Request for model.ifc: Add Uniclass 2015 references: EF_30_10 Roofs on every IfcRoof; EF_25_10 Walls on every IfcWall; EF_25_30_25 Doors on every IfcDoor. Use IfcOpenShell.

First a look at what the model holds.

```python
import ifcopenshell

model = ifcopenshell.open("model.ifc")
print(model.schema)
print("classifications:", [c.Name for c in model.by_type("IfcClassification")])
for ifc_class in ("IfcDoor", "IfcRoof", "IfcStair", "IfcWall", "IfcWindow"):
    print(ifc_class, len(model.by_type(ifc_class)))
```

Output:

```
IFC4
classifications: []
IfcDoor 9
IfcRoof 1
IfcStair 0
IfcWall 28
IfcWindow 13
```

```python
import ifcopenshell
import ifcopenshell.api.classification

model = ifcopenshell.open("model.ifc")

system = ifcopenshell.api.classification.add_classification(model, classification="Uniclass 2015")

codes = {
    "IfcRoof": ("EF_30_10", "Roofs"),
    "IfcWall": ("EF_25_10", "Walls"),
    "IfcDoor": ("EF_25_30_25", "Doors"),
}
for ifc_class, (code, name) in codes.items():
    products = model.by_type(ifc_class)
    ifcopenshell.api.classification.add_reference(
        model, products=products, classification=system, identification=code, name=name
    )
    print(code, len(products))

model.write("model_v2.ifc")
```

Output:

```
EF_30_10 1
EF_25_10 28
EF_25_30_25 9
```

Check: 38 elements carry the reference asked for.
